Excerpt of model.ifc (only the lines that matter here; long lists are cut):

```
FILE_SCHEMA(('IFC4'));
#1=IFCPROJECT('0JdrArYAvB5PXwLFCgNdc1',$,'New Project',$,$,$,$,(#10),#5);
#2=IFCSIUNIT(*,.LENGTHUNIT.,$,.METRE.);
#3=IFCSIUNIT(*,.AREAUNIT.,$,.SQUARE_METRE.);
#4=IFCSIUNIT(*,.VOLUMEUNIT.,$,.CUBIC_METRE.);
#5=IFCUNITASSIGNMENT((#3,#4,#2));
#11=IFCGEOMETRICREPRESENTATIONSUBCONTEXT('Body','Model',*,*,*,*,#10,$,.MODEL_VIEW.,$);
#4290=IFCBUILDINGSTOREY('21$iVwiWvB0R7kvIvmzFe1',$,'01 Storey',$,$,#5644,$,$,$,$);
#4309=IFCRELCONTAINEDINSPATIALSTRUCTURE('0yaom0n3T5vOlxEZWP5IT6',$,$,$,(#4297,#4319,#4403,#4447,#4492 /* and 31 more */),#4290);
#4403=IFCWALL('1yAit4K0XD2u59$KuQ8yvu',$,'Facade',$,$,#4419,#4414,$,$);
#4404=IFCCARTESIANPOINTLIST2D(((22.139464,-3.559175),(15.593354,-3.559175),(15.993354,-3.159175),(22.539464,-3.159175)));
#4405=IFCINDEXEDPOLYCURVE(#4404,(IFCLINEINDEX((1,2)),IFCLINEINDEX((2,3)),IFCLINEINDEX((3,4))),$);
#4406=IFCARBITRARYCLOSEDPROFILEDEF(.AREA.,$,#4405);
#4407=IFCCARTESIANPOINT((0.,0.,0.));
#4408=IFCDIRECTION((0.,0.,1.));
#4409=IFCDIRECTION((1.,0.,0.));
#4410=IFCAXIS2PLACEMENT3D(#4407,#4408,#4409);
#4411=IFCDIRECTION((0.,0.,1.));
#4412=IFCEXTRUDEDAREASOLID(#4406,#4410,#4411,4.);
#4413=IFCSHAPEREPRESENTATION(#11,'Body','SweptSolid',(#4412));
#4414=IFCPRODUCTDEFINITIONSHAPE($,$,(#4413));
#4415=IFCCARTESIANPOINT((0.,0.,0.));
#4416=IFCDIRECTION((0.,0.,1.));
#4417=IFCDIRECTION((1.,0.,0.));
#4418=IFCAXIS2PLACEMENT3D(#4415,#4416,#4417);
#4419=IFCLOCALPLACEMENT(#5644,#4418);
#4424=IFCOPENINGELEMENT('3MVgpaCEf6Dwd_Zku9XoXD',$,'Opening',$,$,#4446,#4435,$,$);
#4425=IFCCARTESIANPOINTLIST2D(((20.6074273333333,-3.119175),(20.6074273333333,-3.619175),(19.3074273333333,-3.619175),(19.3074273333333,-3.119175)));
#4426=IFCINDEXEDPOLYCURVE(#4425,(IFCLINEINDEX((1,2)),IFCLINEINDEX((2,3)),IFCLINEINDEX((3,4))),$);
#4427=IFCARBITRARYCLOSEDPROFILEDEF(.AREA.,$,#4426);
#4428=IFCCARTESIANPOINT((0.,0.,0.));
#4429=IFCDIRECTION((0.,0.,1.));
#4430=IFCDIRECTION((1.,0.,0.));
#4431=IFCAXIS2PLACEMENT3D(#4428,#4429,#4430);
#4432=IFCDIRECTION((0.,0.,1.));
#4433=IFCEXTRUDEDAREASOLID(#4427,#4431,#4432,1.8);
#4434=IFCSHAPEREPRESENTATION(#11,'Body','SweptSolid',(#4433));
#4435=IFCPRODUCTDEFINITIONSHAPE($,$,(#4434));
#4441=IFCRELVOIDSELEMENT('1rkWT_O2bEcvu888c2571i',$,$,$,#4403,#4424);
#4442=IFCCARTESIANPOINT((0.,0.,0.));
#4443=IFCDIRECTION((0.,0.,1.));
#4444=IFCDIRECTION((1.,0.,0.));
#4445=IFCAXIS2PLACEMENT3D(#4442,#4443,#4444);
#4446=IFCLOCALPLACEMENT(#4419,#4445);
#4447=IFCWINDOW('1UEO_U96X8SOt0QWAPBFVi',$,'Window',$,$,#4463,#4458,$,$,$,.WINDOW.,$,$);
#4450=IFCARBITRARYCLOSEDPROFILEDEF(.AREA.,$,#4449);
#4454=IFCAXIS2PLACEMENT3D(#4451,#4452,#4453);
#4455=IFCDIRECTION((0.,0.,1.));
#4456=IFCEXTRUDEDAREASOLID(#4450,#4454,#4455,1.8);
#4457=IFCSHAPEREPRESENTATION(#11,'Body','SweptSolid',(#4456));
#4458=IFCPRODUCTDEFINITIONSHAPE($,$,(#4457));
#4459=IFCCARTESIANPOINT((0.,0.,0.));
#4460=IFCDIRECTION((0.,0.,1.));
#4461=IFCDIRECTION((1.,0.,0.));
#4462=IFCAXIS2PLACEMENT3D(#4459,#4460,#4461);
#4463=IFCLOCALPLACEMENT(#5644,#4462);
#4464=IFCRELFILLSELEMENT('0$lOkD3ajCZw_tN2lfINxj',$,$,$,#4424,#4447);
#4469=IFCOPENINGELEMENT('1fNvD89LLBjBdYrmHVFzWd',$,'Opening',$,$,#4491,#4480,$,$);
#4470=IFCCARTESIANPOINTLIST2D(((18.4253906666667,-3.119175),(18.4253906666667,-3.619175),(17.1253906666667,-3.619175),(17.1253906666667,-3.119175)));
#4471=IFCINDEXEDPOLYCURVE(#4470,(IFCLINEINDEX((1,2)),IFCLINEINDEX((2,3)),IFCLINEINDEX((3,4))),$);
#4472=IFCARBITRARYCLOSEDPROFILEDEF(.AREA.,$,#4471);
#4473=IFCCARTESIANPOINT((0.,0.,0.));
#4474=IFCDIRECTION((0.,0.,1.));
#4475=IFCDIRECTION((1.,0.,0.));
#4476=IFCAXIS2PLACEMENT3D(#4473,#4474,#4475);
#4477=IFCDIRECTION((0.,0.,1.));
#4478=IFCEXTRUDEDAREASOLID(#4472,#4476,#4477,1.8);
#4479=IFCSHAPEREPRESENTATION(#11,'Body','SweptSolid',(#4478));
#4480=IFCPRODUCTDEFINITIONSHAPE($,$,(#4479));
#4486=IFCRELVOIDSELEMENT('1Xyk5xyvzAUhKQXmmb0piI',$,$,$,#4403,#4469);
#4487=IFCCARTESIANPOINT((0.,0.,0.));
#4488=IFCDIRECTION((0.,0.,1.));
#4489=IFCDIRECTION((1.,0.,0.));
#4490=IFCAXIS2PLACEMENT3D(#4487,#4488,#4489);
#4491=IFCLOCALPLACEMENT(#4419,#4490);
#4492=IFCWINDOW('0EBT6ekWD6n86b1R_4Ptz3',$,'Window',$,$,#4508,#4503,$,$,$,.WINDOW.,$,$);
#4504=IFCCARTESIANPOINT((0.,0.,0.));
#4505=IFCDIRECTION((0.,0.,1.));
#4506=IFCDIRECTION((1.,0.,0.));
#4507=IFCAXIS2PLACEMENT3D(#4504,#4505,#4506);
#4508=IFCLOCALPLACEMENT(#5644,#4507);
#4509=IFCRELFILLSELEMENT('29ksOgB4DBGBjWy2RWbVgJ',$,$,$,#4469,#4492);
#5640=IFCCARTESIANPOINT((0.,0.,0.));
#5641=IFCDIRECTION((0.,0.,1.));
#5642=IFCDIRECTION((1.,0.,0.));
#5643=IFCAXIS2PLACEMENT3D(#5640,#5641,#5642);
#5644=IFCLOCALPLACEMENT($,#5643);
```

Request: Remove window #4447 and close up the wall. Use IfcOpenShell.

```python
import ifcopenshell
import ifcopenshell.api.feature
import ifcopenshell.api.root
import ifcopenshell.geom
import ifcopenshell.util.shape

model = ifcopenshell.open("model.ifc")
settings = ifcopenshell.geom.settings()


def volume(element):
    """Net volume in cubic metres, openings subtracted."""
    shape = ifcopenshell.geom.create_shape(settings, element)
    return ifcopenshell.util.shape.get_volume(shape.geometry)


window = model.by_guid("1UEO_U96X8SOt0QWAPBFVi")
opening = window.FillsVoids[0].RelatingOpeningElement
wall = opening.VoidsElements[0].RelatingBuildingElement
before = volume(wall)

ifcopenshell.api.root.remove_product(model, product=window)
ifcopenshell.api.feature.remove_feature(model, feature=opening)

after = volume(wall)

print(f"wall volume {before:.3f} -> {after:.3f} m3")

model.write("model_updated.ifc")
```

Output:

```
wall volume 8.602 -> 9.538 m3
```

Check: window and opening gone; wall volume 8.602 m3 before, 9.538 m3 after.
